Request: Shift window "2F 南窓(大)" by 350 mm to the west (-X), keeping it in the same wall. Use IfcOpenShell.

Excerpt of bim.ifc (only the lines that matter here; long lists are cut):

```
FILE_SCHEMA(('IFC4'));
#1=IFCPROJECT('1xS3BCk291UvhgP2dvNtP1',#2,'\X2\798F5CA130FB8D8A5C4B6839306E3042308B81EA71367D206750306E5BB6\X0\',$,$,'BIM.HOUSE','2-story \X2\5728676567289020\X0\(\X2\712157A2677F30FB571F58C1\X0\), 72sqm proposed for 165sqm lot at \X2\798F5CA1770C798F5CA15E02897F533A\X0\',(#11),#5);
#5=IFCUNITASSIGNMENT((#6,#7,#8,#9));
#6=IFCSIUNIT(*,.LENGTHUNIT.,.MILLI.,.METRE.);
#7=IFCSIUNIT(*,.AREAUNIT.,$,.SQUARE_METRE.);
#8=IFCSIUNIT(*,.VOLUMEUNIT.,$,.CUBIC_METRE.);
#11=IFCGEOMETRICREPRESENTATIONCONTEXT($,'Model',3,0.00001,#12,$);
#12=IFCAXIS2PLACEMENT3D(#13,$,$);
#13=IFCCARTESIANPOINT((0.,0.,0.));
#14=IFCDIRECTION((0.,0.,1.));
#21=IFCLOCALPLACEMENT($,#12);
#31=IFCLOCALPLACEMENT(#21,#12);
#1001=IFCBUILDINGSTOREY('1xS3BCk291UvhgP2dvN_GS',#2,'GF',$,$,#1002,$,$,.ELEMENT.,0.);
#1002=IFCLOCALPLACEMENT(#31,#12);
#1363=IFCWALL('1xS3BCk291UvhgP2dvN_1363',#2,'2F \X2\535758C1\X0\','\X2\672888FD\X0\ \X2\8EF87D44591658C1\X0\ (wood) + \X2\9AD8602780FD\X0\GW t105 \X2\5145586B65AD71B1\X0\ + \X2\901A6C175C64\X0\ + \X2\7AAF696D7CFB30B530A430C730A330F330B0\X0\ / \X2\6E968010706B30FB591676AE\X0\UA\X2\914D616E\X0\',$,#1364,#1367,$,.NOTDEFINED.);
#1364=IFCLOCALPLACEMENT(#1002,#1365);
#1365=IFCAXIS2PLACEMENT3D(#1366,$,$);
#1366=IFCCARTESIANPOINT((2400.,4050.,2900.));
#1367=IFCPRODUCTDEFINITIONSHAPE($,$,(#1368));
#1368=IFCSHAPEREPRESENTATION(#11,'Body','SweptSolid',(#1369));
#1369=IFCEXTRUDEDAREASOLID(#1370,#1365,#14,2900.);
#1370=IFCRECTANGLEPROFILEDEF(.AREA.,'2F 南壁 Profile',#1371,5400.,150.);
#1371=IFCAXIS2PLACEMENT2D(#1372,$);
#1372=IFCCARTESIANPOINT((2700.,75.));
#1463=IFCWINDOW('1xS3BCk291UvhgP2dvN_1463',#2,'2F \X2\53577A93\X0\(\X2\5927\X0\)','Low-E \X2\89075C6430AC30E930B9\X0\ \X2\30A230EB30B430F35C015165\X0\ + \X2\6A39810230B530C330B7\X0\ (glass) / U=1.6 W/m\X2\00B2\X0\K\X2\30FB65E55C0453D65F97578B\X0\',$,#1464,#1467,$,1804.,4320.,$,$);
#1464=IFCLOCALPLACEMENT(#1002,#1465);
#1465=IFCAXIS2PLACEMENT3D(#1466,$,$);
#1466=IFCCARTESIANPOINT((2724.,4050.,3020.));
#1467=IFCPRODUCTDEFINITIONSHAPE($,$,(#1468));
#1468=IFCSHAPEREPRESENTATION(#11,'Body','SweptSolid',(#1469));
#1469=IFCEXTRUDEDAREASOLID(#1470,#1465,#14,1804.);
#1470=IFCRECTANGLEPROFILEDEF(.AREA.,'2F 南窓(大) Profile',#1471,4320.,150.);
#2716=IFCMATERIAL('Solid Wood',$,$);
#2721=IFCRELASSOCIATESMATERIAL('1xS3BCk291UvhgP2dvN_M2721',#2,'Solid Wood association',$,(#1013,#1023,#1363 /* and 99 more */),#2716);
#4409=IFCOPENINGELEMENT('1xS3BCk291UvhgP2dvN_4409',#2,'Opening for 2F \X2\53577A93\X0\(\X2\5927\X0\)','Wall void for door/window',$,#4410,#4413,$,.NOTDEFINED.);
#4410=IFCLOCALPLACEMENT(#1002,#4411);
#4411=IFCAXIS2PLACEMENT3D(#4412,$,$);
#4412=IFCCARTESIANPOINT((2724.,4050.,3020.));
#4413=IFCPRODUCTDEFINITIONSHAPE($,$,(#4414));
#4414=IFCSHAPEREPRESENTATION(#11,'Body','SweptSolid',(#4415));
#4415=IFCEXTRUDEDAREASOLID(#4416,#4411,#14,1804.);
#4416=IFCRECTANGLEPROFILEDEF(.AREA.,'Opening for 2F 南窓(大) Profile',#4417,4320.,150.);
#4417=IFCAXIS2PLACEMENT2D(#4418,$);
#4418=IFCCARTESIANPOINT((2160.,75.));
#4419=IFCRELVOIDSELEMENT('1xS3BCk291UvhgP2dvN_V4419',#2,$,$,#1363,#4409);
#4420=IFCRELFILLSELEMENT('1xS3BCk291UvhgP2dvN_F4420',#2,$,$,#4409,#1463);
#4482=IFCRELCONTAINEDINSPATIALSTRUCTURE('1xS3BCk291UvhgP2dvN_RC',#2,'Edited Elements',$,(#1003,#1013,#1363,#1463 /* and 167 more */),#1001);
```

```python
import ifcopenshell
import ifcopenshell.api.geometry
import ifcopenshell.util.placement

model = ifcopenshell.open("bim.ifc")

window = model.by_guid("1xS3BCk291UvhgP2dvN_1463")
opening = window.FillsVoids[0].RelatingOpeningElement
wall = opening.VoidsElements[0].RelatingBuildingElement

wall_matrix = ifcopenshell.util.placement.get_local_placement(wall.ObjectPlacement)
shift = wall_matrix[:3, 0] * -350.0
before = ifcopenshell.util.placement.get_local_placement(window.ObjectPlacement)[:3, 3].copy()

# The window is not placed relative to its opening, so move both.
for product in (opening, window):
    matrix = ifcopenshell.util.placement.get_local_placement(product.ObjectPlacement)
    matrix[:3, 3] += shift
    ifcopenshell.api.geometry.edit_object_placement(model, product=product, matrix=matrix, is_si=False)

after = ifcopenshell.util.placement.get_local_placement(window.ObjectPlacement)[:3, 3]
print("window moved by", (after - before).round(3) + 0.0)

model.write("bim_edited.ifc")
```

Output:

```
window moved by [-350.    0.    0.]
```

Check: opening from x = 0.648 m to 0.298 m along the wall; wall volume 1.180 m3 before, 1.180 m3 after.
